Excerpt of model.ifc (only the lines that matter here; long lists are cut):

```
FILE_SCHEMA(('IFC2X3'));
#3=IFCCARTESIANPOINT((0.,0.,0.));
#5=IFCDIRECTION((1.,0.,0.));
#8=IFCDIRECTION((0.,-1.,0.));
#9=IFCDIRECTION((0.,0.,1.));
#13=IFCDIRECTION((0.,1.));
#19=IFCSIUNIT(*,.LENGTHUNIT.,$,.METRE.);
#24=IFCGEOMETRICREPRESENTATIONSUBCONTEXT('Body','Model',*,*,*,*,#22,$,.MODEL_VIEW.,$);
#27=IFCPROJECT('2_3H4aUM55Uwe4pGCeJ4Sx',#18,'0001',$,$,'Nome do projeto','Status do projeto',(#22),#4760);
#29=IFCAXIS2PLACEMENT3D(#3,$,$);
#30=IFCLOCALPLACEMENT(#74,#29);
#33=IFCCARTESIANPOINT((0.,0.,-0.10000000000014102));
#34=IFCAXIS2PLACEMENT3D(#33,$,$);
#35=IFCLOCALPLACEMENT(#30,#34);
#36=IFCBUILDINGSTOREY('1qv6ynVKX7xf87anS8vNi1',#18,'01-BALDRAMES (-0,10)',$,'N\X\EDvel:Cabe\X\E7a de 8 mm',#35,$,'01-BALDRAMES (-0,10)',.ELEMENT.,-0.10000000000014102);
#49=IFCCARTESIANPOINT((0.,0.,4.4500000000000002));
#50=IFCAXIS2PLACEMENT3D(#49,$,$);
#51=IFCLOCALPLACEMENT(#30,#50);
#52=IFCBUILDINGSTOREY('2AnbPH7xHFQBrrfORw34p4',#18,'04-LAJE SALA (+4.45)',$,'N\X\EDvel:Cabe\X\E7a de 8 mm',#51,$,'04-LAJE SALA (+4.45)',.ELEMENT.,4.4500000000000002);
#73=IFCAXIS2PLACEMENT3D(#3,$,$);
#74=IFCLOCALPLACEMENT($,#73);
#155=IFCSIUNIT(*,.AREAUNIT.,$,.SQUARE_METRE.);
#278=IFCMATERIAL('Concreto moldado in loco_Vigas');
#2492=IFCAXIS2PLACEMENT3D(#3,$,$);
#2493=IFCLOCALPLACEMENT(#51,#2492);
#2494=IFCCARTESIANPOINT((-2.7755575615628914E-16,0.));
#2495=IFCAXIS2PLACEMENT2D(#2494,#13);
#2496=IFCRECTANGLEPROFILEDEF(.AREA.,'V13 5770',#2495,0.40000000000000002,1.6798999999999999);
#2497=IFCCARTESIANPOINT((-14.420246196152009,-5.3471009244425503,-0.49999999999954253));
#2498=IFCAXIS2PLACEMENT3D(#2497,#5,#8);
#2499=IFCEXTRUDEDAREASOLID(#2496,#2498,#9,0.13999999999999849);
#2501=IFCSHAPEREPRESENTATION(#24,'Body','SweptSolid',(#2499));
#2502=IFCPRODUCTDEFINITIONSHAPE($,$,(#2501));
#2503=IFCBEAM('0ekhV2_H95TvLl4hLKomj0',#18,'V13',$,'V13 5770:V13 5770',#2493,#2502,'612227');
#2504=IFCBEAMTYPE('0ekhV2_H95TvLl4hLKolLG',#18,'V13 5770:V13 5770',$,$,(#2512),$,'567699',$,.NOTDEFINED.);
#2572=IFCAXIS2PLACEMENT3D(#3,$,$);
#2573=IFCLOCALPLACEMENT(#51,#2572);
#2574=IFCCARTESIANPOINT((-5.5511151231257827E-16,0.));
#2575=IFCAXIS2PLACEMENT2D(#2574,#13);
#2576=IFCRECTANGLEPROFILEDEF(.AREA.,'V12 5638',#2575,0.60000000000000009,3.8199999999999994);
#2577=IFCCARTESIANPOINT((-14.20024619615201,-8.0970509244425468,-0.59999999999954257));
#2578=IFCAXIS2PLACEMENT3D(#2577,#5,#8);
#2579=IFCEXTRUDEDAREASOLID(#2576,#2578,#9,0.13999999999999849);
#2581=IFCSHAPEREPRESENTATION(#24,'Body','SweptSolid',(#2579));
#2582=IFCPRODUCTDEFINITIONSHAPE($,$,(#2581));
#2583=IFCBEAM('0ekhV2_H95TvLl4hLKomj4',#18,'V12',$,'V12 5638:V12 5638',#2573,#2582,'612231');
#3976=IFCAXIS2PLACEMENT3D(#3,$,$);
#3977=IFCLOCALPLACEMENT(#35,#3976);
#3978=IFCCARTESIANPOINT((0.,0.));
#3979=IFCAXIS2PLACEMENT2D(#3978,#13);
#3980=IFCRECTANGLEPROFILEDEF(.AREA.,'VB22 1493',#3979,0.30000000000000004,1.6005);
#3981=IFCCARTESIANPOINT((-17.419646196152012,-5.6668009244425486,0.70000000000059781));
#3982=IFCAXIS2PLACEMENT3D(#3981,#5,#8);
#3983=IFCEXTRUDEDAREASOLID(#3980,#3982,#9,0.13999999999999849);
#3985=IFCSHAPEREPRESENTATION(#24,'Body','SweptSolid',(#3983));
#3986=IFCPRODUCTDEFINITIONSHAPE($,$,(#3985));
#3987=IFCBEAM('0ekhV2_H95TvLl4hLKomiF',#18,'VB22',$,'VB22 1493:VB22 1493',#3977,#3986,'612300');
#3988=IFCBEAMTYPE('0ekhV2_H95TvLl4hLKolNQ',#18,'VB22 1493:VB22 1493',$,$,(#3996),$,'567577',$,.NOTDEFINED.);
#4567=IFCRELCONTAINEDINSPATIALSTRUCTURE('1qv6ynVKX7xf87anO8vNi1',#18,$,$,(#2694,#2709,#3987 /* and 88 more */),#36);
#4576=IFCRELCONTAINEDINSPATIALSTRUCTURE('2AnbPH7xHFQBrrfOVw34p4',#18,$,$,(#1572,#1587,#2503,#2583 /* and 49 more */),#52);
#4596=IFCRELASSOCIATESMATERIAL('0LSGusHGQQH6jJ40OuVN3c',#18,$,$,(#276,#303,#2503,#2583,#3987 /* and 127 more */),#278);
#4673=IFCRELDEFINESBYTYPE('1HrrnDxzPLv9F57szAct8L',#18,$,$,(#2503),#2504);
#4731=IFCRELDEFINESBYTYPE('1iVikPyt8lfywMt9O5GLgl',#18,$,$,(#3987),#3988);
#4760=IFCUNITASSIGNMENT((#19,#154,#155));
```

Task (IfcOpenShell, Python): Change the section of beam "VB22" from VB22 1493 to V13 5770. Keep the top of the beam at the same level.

```python
import ifcopenshell
import ifcopenshell.api.type
import ifcopenshell.util.element
import ifcopenshell.util.representation

model = ifcopenshell.open("model.ifc")

member = model.by_guid("0ekhV2_H95TvLl4hLKomiF")
source = next(p for p in model.by_type("IfcRectangleProfileDef") if p.ProfileName == "V13 5770")

body = ifcopenshell.util.representation.get_representation(member, "Model", "Body")
solid = body.Items[0]
old_profile = solid.SweptArea

# Copy the section's sizes but keep this member's own profile position.
profile = ifcopenshell.util.element.copy(model, source)
# Profiles are centred, so shift by half the change in depth to hold the top.
shift = (old_profile.XDim - profile.XDim) / 2
x, y = old_profile.Position.Location.Coordinates
up = (0.0, -1.0)  # upwards, in the solid's own plane
location = model.createIfcCartesianPoint((x + up[0] * shift, y + up[1] * shift))
profile.Position = model.createIfcAxis2Placement2D(location, old_profile.Position.RefDirection)
solid.SweptArea = profile
if not model.get_total_inverses(old_profile):
    ifcopenshell.util.element.remove_deep2(model, old_profile)

new_type = model.by_guid("0ekhV2_H95TvLl4hLKolLG")
ifcopenshell.api.type.assign_type(
    model, related_objects=[member], relating_type=new_type, should_map_representations=False
)
member.ObjectType = "V13 5770:V13 5770"

print(solid.SweptArea)

model.write("model_rev.ifc")
```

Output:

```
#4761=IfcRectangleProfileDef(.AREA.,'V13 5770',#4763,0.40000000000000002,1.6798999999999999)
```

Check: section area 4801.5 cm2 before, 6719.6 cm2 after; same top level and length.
